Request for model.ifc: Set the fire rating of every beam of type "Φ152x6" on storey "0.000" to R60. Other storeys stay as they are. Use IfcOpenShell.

First a look at what the model holds.

```python
import ifcopenshell
import ifcopenshell.util.element

model = ifcopenshell.open("model.ifc")
print(model.schema)
storey = next(s for s in model.by_type("IfcBuildingStorey") if s.Name == "0.000")
beams = [e for e in ifcopenshell.util.element.get_decomposition(storey) if e.is_a("IfcBeam")]
seen = {}
for e in beams:
    element_type = ifcopenshell.util.element.get_type(e)
    key = (element_type.Name if element_type != e and element_type else None, ifcopenshell.util.element.get_pset(e, "Pset_BeamCommon", "FireRating"))
    seen[key] = seen.get(key, 0) + 1
for (name, value), count in sorted(seen.items(), key=str):
    print(count, "x", name, "|", value)
```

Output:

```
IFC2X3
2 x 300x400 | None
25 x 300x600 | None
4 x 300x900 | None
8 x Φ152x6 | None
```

```python
import ifcopenshell
import ifcopenshell.api.pset
import ifcopenshell.util.element

model = ifcopenshell.open("model.ifc")

storey = next(s for s in model.by_type("IfcBuildingStorey") if s.Name == "0.000")
beams = [e for e in ifcopenshell.util.element.get_decomposition(storey) if e.is_a("IfcBeam")]

count = 0
for e in beams:
    element_type = ifcopenshell.util.element.get_type(e)
    if element_type in (None, e) or element_type.Name != "Φ152x6":
        continue
    # add_pset returns the element's existing set when there is one.
    pset = ifcopenshell.api.pset.add_pset(model, product=e, name="Pset_BeamCommon")
    ifcopenshell.api.pset.edit_pset(model, pset=pset, properties={"FireRating": "R60"})
    count += 1

print(count, "beams updated")

model.write("model_edited.ifc")
```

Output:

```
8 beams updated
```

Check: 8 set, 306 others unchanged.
